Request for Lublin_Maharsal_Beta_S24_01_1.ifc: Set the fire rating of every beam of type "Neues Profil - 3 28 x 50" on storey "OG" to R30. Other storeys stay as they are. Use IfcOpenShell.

First a look at what the model holds.

```python
import ifcopenshell
import ifcopenshell.util.element

model = ifcopenshell.open("Lublin_Maharsal_Beta_S24_01_1.ifc")
print(model.schema)
storey = next(s for s in model.by_type("IfcBuildingStorey") if s.Name == "OG")
beams = [e for e in ifcopenshell.util.element.get_decomposition(storey) if e.is_a("IfcBeam")]
seen = {}
for e in beams:
    element_type = ifcopenshell.util.element.get_type(e)
    key = (element_type.Name if element_type != e and element_type else None, ifcopenshell.util.element.get_pset(e, "Pset_BeamCommon", "FireRating"))
    seen[key] = seen.get(key, 0) + 1
for (name, value), count in sorted(seen.items(), key=str):
    print(count, "x", name, "|", value)
```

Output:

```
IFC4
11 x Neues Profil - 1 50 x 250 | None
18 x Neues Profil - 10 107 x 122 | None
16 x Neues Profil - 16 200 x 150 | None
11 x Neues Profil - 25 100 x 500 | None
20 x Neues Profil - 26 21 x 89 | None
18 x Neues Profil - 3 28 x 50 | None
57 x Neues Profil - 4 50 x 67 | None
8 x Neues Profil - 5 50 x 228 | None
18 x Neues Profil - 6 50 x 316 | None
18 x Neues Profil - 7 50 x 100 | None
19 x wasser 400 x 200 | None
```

```python
import ifcopenshell
import ifcopenshell.api.pset
import ifcopenshell.util.element

model = ifcopenshell.open("Lublin_Maharsal_Beta_S24_01_1.ifc")

storey = next(s for s in model.by_type("IfcBuildingStorey") if s.Name == "OG")
beams = [e for e in ifcopenshell.util.element.get_decomposition(storey) if e.is_a("IfcBeam")]

count = 0
for e in beams:
    element_type = ifcopenshell.util.element.get_type(e)
    if element_type in (None, e) or element_type.Name != "Neues Profil - 3 28 x 50":
        continue
    # add_pset returns the element's existing set when there is one.
    pset = ifcopenshell.api.pset.add_pset(model, product=e, name="Pset_BeamCommon")
    ifcopenshell.api.pset.edit_pset(model, pset=pset, properties={"FireRating": "R30"})
    count += 1

print(count, "beams updated")

model.write("Lublin_Maharsal_Beta_S24_01_1_rev.ifc")
```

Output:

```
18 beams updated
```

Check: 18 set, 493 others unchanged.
